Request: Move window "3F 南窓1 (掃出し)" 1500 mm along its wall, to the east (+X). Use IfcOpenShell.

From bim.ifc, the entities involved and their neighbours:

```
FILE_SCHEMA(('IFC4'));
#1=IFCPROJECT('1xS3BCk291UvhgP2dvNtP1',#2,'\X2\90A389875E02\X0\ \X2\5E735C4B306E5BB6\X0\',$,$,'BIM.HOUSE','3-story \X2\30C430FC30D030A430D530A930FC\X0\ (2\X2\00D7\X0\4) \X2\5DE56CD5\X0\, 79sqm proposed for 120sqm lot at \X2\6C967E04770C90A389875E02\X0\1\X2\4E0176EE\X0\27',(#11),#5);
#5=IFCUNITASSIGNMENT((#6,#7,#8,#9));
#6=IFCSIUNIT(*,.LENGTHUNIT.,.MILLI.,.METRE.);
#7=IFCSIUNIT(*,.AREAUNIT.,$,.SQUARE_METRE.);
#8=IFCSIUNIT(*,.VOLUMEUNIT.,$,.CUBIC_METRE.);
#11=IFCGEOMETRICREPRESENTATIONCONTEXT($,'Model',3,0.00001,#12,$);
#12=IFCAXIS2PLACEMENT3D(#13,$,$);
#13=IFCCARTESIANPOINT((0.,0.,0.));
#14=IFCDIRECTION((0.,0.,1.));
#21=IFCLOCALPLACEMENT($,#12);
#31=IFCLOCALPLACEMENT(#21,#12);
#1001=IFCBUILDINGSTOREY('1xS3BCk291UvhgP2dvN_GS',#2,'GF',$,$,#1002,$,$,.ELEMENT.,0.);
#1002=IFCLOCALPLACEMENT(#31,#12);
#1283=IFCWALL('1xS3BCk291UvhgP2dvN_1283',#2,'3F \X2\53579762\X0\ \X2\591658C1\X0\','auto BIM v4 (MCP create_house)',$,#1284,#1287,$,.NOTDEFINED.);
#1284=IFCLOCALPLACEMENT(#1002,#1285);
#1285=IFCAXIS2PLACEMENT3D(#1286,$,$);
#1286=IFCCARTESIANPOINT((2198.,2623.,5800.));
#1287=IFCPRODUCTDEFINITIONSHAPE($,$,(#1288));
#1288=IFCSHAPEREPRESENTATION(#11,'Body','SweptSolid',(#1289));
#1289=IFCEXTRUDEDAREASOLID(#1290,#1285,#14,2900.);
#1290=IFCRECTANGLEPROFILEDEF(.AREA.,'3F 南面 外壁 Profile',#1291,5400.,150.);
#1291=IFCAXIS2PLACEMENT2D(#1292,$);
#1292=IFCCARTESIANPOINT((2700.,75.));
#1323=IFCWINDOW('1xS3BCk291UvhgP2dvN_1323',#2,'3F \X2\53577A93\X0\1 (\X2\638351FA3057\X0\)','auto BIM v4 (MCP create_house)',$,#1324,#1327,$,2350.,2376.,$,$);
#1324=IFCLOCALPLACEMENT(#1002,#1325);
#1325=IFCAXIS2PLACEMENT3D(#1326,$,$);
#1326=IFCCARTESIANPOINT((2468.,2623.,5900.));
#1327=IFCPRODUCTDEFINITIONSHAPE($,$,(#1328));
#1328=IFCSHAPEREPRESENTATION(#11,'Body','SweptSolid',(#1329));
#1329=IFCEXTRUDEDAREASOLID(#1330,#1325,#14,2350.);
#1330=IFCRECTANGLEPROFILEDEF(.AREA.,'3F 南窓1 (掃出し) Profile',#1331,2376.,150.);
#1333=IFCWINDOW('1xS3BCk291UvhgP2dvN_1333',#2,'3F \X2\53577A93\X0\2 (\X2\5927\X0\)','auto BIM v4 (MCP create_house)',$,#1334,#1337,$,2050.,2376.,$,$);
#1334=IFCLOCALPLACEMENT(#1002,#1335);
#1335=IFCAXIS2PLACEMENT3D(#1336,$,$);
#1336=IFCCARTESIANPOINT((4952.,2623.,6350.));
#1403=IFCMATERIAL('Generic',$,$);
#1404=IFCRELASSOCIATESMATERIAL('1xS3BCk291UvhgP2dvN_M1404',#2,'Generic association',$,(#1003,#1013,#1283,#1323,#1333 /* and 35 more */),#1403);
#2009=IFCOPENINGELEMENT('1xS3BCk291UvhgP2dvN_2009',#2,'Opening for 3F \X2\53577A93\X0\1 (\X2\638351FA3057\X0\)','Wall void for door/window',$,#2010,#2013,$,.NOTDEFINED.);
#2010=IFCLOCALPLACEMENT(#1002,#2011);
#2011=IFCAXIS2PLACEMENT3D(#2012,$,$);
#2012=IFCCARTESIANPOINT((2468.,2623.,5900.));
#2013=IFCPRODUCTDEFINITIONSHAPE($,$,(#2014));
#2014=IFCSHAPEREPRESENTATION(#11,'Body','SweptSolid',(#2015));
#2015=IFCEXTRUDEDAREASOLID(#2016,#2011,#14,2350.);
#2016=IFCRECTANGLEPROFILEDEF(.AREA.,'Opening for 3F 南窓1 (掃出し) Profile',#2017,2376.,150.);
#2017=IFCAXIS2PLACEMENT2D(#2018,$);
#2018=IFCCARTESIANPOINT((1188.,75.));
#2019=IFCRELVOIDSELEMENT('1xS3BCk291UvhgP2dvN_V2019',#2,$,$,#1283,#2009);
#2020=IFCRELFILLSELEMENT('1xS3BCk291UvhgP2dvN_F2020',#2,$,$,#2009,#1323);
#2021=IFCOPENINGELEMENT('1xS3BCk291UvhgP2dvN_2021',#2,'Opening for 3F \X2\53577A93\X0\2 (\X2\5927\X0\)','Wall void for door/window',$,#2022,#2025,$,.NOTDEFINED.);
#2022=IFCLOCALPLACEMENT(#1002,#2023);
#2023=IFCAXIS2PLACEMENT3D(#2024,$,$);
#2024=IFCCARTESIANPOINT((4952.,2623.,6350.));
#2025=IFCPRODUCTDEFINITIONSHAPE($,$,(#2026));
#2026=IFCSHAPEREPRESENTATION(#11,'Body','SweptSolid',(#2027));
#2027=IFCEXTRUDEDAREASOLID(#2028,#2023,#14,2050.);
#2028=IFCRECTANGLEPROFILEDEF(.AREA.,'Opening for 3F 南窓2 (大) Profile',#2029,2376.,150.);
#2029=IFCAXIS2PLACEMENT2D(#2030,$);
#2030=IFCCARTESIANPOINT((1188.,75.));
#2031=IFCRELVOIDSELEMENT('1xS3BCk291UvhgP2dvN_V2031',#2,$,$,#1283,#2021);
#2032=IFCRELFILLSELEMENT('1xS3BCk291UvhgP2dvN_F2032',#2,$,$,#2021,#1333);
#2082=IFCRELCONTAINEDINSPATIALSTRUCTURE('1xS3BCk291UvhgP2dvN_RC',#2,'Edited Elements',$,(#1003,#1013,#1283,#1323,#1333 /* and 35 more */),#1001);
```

```python
import ifcopenshell
import ifcopenshell.api.geometry
import ifcopenshell.util.placement
import ifcopenshell.util.unit

model = ifcopenshell.open("bim.ifc")
unit_scale = ifcopenshell.util.unit.calculate_unit_scale(model)

window = model.by_guid("1xS3BCk291UvhgP2dvN_1323")
opening = window.FillsVoids[0].RelatingOpeningElement
wall = opening.VoidsElements[0].RelatingBuildingElement

wall_matrix = ifcopenshell.util.placement.get_local_placement(wall.ObjectPlacement)
shift = wall_matrix[:3, 0] * 1.5 / unit_scale
before = ifcopenshell.util.placement.get_local_placement(window.ObjectPlacement)[:3, 3].copy()

# The window is not placed relative to its opening, so move both.
for product in (opening, window):
    matrix = ifcopenshell.util.placement.get_local_placement(product.ObjectPlacement)
    matrix[:3, 3] += shift
    ifcopenshell.api.geometry.edit_object_placement(model, product=product, matrix=matrix, is_si=False)

after = ifcopenshell.util.placement.get_local_placement(window.ObjectPlacement)[:3, 3]
print("window moved by", (after - before).round(3) + 0.0)

model.write("bim_edited.ifc")
```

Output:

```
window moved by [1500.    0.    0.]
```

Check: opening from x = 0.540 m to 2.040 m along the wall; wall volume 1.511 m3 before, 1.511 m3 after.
